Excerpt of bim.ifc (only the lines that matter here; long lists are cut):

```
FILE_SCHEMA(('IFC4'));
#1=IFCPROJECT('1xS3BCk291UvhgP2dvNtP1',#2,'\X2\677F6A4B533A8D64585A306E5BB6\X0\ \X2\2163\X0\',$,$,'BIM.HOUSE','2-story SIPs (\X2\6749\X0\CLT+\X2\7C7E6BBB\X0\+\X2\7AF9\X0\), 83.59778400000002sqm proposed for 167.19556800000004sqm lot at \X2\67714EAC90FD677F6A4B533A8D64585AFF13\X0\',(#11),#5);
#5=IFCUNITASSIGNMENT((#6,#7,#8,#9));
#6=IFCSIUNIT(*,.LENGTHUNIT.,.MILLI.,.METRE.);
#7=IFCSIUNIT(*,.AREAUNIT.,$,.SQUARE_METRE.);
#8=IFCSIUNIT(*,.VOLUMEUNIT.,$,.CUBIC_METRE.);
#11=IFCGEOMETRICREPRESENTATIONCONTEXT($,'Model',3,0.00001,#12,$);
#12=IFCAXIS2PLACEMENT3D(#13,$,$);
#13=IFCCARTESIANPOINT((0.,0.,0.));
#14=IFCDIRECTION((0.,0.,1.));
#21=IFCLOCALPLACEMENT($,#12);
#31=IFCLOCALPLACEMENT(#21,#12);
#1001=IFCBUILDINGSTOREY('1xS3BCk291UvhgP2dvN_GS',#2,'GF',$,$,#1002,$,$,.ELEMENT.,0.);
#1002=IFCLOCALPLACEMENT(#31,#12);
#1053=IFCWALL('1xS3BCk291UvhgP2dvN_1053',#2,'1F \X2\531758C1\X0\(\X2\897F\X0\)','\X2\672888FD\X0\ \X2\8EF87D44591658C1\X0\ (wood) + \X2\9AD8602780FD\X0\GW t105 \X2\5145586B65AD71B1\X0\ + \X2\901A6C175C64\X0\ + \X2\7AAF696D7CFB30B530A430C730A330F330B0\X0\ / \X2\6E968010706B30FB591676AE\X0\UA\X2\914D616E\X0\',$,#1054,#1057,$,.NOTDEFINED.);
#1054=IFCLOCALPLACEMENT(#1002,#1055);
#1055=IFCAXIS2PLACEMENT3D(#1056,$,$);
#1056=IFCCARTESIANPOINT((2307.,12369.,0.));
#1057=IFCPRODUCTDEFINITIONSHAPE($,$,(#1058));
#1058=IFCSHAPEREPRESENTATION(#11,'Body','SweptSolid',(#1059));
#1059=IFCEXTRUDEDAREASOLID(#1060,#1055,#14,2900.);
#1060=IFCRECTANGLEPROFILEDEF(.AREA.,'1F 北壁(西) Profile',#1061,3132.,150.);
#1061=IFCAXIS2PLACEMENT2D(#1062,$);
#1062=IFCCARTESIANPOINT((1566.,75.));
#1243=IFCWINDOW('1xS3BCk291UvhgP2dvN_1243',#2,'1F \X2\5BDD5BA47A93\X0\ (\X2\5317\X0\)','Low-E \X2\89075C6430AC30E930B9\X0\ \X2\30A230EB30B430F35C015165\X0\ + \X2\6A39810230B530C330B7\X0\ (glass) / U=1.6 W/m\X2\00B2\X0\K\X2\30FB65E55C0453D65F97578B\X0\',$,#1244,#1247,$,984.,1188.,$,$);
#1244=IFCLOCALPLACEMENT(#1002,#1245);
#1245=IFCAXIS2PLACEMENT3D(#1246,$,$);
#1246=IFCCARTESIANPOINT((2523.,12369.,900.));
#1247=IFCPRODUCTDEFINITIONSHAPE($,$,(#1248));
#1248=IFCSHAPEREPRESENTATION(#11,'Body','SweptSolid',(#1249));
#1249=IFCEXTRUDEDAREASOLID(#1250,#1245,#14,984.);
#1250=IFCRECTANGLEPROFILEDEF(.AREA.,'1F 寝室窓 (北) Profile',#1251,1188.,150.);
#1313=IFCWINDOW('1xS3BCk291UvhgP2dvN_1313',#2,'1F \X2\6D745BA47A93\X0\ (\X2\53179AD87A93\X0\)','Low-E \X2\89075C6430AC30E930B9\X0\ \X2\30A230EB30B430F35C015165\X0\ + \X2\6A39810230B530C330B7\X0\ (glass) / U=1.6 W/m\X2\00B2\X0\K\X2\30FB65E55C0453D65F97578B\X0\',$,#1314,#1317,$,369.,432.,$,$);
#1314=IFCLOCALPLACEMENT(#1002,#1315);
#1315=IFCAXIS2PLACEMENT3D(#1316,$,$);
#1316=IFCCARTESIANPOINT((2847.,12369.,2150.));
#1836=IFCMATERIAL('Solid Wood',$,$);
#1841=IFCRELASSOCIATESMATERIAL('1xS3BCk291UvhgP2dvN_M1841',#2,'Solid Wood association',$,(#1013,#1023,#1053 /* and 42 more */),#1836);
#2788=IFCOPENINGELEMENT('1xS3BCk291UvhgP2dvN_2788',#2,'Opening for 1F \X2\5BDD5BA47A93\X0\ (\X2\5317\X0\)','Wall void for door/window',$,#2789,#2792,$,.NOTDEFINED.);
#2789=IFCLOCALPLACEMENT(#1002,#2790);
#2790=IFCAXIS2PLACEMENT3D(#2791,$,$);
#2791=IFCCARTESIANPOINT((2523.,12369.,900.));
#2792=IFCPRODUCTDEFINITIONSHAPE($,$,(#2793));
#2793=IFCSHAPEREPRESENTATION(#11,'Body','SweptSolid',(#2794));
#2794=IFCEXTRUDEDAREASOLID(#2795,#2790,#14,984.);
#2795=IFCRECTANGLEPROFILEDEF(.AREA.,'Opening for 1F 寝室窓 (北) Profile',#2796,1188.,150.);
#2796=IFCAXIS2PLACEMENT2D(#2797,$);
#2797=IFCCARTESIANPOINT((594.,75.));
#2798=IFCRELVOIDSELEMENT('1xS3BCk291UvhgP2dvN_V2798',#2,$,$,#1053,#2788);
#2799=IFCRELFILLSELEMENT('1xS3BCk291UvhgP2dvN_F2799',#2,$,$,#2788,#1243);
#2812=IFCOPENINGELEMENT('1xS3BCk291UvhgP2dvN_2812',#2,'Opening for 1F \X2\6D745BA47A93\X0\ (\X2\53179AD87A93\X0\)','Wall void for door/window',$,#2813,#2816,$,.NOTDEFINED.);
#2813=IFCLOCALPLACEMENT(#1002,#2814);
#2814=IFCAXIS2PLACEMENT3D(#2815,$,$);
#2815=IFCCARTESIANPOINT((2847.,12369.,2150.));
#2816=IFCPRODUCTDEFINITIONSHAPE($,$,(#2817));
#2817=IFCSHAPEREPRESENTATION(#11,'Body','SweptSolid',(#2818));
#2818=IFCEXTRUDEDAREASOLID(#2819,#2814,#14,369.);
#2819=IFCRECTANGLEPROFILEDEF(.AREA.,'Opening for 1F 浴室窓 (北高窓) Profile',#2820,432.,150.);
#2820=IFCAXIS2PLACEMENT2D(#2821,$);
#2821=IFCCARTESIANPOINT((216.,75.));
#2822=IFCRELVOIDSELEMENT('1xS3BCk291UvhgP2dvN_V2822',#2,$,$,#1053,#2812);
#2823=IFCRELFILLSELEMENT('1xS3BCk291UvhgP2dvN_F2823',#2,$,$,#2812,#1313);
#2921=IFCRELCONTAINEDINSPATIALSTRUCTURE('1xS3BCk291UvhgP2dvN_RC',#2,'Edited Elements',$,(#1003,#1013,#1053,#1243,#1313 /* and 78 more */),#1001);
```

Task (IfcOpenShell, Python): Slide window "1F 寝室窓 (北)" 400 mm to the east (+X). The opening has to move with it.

```python
import ifcopenshell
import ifcopenshell.api.geometry
import ifcopenshell.util.placement
import ifcopenshell.util.unit

model = ifcopenshell.open("bim.ifc")
unit_scale = ifcopenshell.util.unit.calculate_unit_scale(model)

window = model.by_guid("1xS3BCk291UvhgP2dvN_1243")
opening = window.FillsVoids[0].RelatingOpeningElement
wall = opening.VoidsElements[0].RelatingBuildingElement

wall_matrix = ifcopenshell.util.placement.get_local_placement(wall.ObjectPlacement)
shift = wall_matrix[:3, 0] * 0.4 / unit_scale
before = ifcopenshell.util.placement.get_local_placement(window.ObjectPlacement)[:3, 3].copy()

# The window is not placed relative to its opening, so move both.
for product in (opening, window):
    matrix = ifcopenshell.util.placement.get_local_placement(product.ObjectPlacement)
    matrix[:3, 3] += shift
    ifcopenshell.api.geometry.edit_object_placement(model, product=product, matrix=matrix, is_si=False)

after = ifcopenshell.util.placement.get_local_placement(window.ObjectPlacement)[:3, 3]
print("window moved by", (after - before).round(3) + 0.0)

model.write("bim_v2.ifc")
```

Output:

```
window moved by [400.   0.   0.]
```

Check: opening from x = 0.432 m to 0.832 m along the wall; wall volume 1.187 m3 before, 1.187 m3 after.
